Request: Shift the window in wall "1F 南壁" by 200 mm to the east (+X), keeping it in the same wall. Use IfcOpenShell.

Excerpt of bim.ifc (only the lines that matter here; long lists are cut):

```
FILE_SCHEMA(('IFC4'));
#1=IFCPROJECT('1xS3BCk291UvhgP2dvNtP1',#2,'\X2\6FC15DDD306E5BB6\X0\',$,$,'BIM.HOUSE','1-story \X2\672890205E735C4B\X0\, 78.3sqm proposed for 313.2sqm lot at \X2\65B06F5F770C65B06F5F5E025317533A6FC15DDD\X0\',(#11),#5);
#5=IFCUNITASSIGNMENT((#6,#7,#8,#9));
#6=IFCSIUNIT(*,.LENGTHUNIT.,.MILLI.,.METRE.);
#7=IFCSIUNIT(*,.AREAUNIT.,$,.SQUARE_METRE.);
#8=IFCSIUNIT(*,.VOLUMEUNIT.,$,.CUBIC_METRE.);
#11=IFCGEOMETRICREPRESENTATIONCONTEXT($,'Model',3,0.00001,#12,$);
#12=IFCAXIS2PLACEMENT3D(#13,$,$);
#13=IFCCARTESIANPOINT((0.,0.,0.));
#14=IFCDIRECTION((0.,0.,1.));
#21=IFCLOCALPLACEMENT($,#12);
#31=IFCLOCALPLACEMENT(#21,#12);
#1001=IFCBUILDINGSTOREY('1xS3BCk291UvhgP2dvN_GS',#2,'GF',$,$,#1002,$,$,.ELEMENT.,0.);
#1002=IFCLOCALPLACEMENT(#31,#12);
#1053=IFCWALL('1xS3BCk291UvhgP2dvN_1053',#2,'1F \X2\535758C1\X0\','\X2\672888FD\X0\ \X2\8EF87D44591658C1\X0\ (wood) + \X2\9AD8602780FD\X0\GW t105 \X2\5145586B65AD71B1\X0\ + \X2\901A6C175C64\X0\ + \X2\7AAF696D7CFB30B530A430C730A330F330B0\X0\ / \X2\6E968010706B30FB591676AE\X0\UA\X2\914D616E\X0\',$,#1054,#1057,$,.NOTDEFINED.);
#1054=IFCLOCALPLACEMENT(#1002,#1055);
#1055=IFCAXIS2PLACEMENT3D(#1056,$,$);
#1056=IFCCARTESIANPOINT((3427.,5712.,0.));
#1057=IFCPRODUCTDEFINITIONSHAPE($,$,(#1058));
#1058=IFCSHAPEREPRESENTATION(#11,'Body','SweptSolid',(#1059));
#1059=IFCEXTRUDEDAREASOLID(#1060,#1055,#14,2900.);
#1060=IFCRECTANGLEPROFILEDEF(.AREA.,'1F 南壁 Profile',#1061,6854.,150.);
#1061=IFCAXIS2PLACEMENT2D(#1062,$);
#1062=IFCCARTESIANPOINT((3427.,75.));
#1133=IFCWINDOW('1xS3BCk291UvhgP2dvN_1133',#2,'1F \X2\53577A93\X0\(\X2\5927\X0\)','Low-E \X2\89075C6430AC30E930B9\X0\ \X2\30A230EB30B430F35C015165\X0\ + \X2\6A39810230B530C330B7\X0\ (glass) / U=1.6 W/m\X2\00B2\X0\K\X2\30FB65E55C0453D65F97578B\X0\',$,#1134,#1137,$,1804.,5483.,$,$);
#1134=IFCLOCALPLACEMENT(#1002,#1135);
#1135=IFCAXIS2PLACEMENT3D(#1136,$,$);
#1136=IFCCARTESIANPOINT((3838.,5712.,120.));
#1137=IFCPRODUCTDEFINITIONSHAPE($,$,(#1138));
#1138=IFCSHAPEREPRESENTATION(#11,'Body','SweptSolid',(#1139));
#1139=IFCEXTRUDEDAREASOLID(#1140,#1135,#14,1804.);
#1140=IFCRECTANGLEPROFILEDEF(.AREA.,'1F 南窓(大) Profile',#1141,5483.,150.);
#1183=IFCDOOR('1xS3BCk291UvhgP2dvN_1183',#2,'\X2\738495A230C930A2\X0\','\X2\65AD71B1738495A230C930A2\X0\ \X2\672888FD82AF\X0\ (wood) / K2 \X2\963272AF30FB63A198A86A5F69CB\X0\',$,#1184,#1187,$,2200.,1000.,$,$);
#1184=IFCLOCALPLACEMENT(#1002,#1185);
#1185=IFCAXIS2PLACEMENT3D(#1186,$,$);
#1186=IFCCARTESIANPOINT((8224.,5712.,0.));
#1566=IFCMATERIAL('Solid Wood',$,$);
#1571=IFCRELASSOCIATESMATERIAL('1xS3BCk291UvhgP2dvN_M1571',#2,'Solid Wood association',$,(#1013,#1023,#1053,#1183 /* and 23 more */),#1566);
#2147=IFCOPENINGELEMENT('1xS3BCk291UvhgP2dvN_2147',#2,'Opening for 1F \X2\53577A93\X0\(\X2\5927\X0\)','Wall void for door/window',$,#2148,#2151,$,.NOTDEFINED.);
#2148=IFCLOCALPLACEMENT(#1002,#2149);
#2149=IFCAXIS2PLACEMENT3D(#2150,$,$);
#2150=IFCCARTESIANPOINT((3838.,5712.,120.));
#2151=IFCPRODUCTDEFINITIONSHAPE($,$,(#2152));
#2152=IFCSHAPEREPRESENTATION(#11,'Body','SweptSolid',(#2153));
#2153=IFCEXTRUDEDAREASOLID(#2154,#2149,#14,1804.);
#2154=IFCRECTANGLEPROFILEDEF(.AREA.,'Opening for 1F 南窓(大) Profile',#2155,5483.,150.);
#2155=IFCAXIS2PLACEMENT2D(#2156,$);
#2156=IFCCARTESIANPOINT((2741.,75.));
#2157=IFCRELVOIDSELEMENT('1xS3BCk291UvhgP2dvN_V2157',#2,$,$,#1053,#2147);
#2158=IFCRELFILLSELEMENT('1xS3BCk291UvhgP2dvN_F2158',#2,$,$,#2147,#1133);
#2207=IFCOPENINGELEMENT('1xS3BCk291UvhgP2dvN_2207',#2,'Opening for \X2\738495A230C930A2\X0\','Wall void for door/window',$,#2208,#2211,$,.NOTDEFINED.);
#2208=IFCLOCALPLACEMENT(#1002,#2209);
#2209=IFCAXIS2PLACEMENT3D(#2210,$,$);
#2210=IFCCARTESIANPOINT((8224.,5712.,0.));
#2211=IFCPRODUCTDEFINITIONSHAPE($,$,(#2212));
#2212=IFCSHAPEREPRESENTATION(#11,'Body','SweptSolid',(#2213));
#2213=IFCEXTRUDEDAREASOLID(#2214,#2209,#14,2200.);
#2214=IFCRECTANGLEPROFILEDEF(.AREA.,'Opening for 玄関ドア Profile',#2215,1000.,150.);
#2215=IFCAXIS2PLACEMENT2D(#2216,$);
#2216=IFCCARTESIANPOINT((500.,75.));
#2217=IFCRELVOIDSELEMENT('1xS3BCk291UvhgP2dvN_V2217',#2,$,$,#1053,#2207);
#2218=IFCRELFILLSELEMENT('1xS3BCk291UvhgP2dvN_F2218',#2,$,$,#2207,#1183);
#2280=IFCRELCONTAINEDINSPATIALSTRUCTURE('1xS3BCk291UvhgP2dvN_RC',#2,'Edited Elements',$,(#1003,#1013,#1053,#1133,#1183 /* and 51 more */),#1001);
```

```python
import ifcopenshell
import ifcopenshell.api.geometry
import ifcopenshell.util.placement
import ifcopenshell.util.unit

model = ifcopenshell.open("bim.ifc")
unit_scale = ifcopenshell.util.unit.calculate_unit_scale(model)

window = model.by_guid("1xS3BCk291UvhgP2dvN_1133")
opening = window.FillsVoids[0].RelatingOpeningElement
wall = opening.VoidsElements[0].RelatingBuildingElement

wall_matrix = ifcopenshell.util.placement.get_local_placement(wall.ObjectPlacement)
shift = wall_matrix[:3, 0] * 0.2 / unit_scale
before = ifcopenshell.util.placement.get_local_placement(window.ObjectPlacement)[:3, 3].copy()

# The window is not placed relative to its opening, so move both.
for product in (opening, window):
    matrix = ifcopenshell.util.placement.get_local_placement(product.ObjectPlacement)
    matrix[:3, 3] += shift
    ifcopenshell.api.geometry.edit_object_placement(model, product=product, matrix=matrix, is_si=False)

after = ifcopenshell.util.placement.get_local_placement(window.ObjectPlacement)[:3, 3]
print("window moved by", (after - before).round(3) + 0.0)

model.write("bim_v2.ifc")
```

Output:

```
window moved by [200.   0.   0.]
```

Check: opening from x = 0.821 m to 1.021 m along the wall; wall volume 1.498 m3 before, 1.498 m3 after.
